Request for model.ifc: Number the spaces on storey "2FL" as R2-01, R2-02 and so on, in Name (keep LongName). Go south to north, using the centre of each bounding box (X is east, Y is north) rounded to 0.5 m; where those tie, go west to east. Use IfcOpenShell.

First a look at what the model holds.

```python
import ifcopenshell
import ifcopenshell.util.element
import ifcopenshell.util.placement

model = ifcopenshell.open("model.ifc")
print(model.schema)
storey = next(s for s in model.by_type("IfcBuildingStorey") if s.Name == "2FL")
spaces = [e for e in ifcopenshell.util.element.get_decomposition(storey) if e.is_a("IfcSpace")]
for e in sorted(spaces, key=lambda e: e.id()):
    origin = ifcopenshell.util.placement.get_local_placement(e.ObjectPlacement)[:3, 3]
    print(e.id(), e.Name, e.LongName, origin.round(2) + 0.0, sep=" | ")
```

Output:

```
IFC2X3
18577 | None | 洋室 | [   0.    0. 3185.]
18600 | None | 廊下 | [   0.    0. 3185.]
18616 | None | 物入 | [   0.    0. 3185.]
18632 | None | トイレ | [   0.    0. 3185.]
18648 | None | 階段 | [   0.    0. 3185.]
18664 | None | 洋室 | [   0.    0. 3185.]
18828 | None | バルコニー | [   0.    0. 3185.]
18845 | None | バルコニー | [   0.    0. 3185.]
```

```python
import ifcopenshell
import ifcopenshell.geom
import ifcopenshell.util.element
import ifcopenshell.util.shape

model = ifcopenshell.open("model.ifc")
settings = ifcopenshell.geom.settings()
settings.set("use-world-coords", True)


def centre(element):
    shape = ifcopenshell.geom.create_shape(settings, element)
    return ifcopenshell.util.shape.get_bbox_centroid(shape.geometry)


storey = next(s for s in model.by_type("IfcBuildingStorey") if s.Name == "2FL")
spaces = [e for e in ifcopenshell.util.element.get_decomposition(storey) if e.is_a("IfcSpace")]

# Insertion points can sit at a corner or the storey origin, so sort by the geometry (in metres).
centres = {e: centre(e) for e in spaces}
spaces.sort(key=lambda e: (round(centres[e][1] / 0.5), centres[e][0]))

for i, e in enumerate(spaces, start=1):
    number = f"R2-{i:02d}"
    e.Name = number
    print(e.id(), number)

model.write("model_v2.ifc")
```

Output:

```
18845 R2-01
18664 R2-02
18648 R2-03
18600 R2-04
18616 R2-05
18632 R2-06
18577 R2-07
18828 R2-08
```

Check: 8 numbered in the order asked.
